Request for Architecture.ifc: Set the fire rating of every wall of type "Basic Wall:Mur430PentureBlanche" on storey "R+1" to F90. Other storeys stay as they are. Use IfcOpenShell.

First a look at what the model holds.

```python
import ifcopenshell
import ifcopenshell.util.element

model = ifcopenshell.open("Architecture.ifc")
print(model.schema)
storey = next(s for s in model.by_type("IfcBuildingStorey") if s.Name == "R+1")
walls = [e for e in ifcopenshell.util.element.get_decomposition(storey) if e.is_a("IfcWall")]
seen = {}
for e in walls:
    element_type = ifcopenshell.util.element.get_type(e)
    key = (element_type.Name if element_type != e and element_type else None, ifcopenshell.util.element.get_pset(e, "Pset_WallCommon", "FireRating"))
    seen[key] = seen.get(key, 0) + 1
for (name, value), count in sorted(seen.items(), key=str):
    print(count, "x", name, "|", value)
```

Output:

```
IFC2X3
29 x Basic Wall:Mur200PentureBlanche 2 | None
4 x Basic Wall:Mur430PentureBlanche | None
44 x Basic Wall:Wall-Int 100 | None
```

```python
import ifcopenshell
import ifcopenshell.api.pset
import ifcopenshell.util.element

model = ifcopenshell.open("Architecture.ifc")

storey = next(s for s in model.by_type("IfcBuildingStorey") if s.Name == "R+1")
walls = [e for e in ifcopenshell.util.element.get_decomposition(storey) if e.is_a("IfcWall")]

count = 0
for e in walls:
    element_type = ifcopenshell.util.element.get_type(e)
    if element_type in (None, e) or element_type.Name != "Basic Wall:Mur430PentureBlanche":
        continue
    # add_pset returns the element's existing set when there is one.
    pset = ifcopenshell.api.pset.add_pset(model, product=e, name="Pset_WallCommon")
    ifcopenshell.api.pset.edit_pset(model, pset=pset, properties={"FireRating": "F90"})
    count += 1

print(count, "walls updated")

model.write("Architecture_rev.ifc")
```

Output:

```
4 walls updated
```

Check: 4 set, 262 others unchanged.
